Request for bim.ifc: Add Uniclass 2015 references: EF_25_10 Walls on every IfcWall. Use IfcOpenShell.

First a look at what the model holds.

```python
import ifcopenshell

model = ifcopenshell.open("bim.ifc")
print(model.schema)
print("classifications:", [c.Name for c in model.by_type("IfcClassification")])
for ifc_class in ("IfcDoor", "IfcRoof", "IfcStair", "IfcWall", "IfcWindow"):
    print(ifc_class, len(model.by_type(ifc_class)))
```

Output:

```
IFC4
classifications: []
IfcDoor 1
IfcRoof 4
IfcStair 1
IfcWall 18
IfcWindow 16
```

```python
import ifcopenshell
import ifcopenshell.api.classification

model = ifcopenshell.open("bim.ifc")

system = ifcopenshell.api.classification.add_classification(model, classification="Uniclass 2015")

codes = {
    "IfcWall": ("EF_25_10", "Walls"),
}
for ifc_class, (code, name) in codes.items():
    products = model.by_type(ifc_class)
    ifcopenshell.api.classification.add_reference(
        model, products=products, classification=system, identification=code, name=name
    )
    print(code, len(products))

model.write("bim-out.ifc")
```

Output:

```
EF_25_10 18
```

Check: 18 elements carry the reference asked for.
